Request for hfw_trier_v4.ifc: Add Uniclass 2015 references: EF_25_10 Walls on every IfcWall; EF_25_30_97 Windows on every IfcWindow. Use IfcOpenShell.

First a look at what the model holds.

```python
import ifcopenshell

model = ifcopenshell.open("hfw_trier_v4.ifc")
print(model.schema)
print("classifications:", [c.Name for c in model.by_type("IfcClassification")])
for ifc_class in ("IfcDoor", "IfcRoof", "IfcStair", "IfcWall", "IfcWindow"):
    print(ifc_class, len(model.by_type(ifc_class)))
```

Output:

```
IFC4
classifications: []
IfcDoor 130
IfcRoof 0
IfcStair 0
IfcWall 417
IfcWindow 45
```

```python
import ifcopenshell
import ifcopenshell.api.classification

model = ifcopenshell.open("hfw_trier_v4.ifc")

system = ifcopenshell.api.classification.add_classification(model, classification="Uniclass 2015")

codes = {
    "IfcWall": ("EF_25_10", "Walls"),
    "IfcWindow": ("EF_25_30_97", "Windows"),
}
for ifc_class, (code, name) in codes.items():
    products = model.by_type(ifc_class)
    ifcopenshell.api.classification.add_reference(
        model, products=products, classification=system, identification=code, name=name
    )
    print(code, len(products))

model.write("hfw_trier_v4_updated.ifc")
```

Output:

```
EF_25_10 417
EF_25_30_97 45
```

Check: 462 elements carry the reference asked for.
